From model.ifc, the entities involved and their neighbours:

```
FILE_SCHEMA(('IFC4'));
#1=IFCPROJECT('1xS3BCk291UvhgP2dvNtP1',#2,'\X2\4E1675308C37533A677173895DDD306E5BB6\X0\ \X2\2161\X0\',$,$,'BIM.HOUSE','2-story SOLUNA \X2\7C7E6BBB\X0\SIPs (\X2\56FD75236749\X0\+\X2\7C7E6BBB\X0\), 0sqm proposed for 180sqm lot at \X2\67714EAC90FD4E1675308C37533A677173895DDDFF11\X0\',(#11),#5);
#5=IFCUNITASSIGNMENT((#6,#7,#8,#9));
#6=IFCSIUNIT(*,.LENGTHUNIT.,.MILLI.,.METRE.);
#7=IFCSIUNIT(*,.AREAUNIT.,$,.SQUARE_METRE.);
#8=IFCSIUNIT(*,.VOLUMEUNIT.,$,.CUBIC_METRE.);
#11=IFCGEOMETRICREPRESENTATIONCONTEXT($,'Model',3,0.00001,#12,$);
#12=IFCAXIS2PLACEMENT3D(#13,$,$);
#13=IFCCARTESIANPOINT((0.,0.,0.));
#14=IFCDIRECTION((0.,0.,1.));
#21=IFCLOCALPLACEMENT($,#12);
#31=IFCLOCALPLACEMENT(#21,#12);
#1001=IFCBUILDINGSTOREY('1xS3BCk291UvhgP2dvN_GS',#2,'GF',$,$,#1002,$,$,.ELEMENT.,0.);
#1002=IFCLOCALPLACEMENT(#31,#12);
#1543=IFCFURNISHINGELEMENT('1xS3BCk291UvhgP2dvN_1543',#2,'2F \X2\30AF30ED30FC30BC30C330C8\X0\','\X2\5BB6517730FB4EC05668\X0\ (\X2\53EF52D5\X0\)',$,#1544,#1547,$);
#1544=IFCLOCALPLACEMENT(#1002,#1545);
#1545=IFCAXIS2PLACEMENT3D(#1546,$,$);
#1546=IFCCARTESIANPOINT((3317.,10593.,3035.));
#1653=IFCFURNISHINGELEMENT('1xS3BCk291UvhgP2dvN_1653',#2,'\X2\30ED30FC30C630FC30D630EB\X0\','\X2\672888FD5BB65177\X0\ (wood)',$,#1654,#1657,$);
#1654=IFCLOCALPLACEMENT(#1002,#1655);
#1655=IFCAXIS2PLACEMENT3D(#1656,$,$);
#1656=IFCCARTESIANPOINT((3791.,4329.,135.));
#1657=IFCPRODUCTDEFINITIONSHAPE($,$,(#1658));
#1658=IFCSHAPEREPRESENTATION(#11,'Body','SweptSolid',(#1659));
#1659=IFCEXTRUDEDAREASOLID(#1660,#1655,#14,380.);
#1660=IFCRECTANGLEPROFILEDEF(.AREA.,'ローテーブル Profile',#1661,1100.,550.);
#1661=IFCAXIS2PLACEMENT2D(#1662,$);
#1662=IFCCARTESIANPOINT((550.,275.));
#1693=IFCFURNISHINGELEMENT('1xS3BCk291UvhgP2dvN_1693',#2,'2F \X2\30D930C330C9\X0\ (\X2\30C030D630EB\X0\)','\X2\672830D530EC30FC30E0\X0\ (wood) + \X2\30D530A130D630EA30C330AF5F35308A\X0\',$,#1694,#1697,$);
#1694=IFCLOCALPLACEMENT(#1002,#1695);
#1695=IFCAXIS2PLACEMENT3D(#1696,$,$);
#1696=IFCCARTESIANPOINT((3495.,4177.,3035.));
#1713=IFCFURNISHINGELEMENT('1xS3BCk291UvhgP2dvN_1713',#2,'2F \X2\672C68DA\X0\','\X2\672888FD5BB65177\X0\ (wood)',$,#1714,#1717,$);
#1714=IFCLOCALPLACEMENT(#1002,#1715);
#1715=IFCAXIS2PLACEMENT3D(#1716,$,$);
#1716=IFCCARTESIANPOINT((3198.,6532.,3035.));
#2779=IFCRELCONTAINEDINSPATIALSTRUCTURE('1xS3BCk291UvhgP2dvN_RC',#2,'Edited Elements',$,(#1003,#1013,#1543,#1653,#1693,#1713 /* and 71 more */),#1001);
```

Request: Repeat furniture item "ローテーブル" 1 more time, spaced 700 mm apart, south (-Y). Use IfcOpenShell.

```python
import numpy as np
import ifcopenshell
import ifcopenshell.api.geometry
import ifcopenshell.api.root
import ifcopenshell.util.element
import ifcopenshell.util.placement

model = ifcopenshell.open("model.ifc")


def reuse_history(source, copy):
    """copy_class also copies each property set's owner history, people and application; keep the originals."""
    for rel in copy.IsDefinedBy:
        if rel.is_a("IfcRelDefinesByProperties") and (history := rel.RelatingPropertyDefinition.OwnerHistory):
            rel.RelatingPropertyDefinition.OwnerHistory = source.OwnerHistory
            ifcopenshell.util.element.remove_deep2(model, history)


source = model.by_id(1653)
base = ifcopenshell.util.placement.get_local_placement(source.ObjectPlacement)
step = np.array([0.0, -1.0, 0.0]) * 700.0

for i in range(1, 2):
    copy = ifcopenshell.api.root.copy_class(model, product=source)
    copy.Representation = ifcopenshell.util.element.copy_deep(
        model, source.Representation, exclude=["IfcGeometricRepresentationContext", "IfcRepresentationMap"]
    )
    reuse_history(source, copy)
    matrix = base.copy()
    matrix[:3, 3] += i * step
    print("added at", matrix[:3, 3].round(3) + 0.0)
    ifcopenshell.api.geometry.edit_object_placement(model, product=copy, matrix=matrix, is_si=False)

model.write("model_edited.ifc")
```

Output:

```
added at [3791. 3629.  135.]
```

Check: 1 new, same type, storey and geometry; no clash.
